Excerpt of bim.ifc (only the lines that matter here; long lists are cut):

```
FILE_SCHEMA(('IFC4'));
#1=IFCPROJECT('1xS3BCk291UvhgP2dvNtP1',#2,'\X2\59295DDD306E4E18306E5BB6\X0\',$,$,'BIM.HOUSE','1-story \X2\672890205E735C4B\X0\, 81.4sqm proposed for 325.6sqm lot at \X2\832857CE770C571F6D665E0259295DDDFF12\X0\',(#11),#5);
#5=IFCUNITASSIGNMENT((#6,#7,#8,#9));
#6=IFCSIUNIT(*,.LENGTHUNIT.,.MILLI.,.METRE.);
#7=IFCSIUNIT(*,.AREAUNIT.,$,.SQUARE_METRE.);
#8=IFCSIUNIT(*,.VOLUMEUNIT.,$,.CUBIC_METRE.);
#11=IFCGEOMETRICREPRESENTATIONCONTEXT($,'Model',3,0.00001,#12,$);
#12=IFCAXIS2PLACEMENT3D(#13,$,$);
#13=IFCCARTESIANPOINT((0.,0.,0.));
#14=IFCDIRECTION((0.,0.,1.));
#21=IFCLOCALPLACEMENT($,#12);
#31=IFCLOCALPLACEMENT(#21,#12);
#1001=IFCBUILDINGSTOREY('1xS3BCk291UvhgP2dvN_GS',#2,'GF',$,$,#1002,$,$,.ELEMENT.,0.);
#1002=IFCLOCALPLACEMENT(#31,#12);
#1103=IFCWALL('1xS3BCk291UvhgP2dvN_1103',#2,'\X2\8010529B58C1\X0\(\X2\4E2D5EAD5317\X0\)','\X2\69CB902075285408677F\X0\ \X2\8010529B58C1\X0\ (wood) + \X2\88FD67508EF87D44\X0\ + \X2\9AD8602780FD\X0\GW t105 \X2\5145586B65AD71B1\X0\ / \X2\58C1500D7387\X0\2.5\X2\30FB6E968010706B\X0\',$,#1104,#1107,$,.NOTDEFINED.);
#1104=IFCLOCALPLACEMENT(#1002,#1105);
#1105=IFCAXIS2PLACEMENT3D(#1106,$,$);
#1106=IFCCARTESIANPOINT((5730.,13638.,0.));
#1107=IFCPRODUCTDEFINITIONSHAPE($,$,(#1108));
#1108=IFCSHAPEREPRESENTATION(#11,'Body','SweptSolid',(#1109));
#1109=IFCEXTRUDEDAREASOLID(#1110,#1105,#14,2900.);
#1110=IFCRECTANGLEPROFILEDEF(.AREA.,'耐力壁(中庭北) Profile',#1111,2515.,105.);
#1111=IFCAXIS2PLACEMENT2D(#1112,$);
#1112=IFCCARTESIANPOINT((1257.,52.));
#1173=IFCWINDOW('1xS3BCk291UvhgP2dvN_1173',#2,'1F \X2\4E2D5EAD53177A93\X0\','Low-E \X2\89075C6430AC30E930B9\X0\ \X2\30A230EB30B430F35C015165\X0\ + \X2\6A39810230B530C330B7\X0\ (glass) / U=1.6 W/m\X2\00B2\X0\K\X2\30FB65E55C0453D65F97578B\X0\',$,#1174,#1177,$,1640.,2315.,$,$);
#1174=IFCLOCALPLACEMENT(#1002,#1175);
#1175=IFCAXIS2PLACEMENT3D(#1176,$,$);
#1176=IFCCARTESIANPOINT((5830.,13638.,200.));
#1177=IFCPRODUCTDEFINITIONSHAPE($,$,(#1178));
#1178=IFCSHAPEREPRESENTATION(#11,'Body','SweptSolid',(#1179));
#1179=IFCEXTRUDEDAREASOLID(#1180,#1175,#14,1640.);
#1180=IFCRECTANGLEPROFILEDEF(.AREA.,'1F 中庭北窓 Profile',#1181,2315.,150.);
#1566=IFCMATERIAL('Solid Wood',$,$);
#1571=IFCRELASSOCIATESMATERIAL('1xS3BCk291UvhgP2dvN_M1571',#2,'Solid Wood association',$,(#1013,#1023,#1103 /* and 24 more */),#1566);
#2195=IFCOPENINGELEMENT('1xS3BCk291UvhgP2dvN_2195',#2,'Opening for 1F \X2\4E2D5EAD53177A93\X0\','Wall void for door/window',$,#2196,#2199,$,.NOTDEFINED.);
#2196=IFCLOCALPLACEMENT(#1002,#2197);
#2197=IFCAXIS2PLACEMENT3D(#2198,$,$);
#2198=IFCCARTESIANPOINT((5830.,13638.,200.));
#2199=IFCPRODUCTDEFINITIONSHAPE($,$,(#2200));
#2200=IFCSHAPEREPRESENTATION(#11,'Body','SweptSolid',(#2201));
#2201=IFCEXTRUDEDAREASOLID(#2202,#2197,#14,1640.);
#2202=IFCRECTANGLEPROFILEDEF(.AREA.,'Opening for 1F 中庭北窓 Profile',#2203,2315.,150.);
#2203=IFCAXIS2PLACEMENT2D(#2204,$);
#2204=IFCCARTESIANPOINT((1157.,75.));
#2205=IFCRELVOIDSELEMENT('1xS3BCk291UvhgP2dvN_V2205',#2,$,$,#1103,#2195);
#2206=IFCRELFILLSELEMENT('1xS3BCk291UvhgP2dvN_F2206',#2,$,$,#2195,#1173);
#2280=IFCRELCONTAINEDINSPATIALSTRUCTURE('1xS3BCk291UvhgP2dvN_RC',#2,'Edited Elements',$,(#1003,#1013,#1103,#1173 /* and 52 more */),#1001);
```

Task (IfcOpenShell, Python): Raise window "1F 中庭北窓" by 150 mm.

```python
import numpy as np
import ifcopenshell
import ifcopenshell.api.geometry
import ifcopenshell.util.placement
import ifcopenshell.util.unit

model = ifcopenshell.open("bim.ifc")
unit_scale = ifcopenshell.util.unit.calculate_unit_scale(model)

window = model.by_id(1173)
opening = window.FillsVoids[0].RelatingOpeningElement
dz = 0.15 / unit_scale

shift = np.array([0.0, 0.0, dz])
# The window is not placed relative to its opening, so move both.
for product in (opening, window):
    matrix = ifcopenshell.util.placement.get_local_placement(product.ObjectPlacement)
    matrix[:3, 3] += shift
    ifcopenshell.api.geometry.edit_object_placement(model, product=product, matrix=matrix, is_si=False)

print(f"moved by {dz * unit_scale:+.3f} m")

model.write("bim_updated.ifc")
```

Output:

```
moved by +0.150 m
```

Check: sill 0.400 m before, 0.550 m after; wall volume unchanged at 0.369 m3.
